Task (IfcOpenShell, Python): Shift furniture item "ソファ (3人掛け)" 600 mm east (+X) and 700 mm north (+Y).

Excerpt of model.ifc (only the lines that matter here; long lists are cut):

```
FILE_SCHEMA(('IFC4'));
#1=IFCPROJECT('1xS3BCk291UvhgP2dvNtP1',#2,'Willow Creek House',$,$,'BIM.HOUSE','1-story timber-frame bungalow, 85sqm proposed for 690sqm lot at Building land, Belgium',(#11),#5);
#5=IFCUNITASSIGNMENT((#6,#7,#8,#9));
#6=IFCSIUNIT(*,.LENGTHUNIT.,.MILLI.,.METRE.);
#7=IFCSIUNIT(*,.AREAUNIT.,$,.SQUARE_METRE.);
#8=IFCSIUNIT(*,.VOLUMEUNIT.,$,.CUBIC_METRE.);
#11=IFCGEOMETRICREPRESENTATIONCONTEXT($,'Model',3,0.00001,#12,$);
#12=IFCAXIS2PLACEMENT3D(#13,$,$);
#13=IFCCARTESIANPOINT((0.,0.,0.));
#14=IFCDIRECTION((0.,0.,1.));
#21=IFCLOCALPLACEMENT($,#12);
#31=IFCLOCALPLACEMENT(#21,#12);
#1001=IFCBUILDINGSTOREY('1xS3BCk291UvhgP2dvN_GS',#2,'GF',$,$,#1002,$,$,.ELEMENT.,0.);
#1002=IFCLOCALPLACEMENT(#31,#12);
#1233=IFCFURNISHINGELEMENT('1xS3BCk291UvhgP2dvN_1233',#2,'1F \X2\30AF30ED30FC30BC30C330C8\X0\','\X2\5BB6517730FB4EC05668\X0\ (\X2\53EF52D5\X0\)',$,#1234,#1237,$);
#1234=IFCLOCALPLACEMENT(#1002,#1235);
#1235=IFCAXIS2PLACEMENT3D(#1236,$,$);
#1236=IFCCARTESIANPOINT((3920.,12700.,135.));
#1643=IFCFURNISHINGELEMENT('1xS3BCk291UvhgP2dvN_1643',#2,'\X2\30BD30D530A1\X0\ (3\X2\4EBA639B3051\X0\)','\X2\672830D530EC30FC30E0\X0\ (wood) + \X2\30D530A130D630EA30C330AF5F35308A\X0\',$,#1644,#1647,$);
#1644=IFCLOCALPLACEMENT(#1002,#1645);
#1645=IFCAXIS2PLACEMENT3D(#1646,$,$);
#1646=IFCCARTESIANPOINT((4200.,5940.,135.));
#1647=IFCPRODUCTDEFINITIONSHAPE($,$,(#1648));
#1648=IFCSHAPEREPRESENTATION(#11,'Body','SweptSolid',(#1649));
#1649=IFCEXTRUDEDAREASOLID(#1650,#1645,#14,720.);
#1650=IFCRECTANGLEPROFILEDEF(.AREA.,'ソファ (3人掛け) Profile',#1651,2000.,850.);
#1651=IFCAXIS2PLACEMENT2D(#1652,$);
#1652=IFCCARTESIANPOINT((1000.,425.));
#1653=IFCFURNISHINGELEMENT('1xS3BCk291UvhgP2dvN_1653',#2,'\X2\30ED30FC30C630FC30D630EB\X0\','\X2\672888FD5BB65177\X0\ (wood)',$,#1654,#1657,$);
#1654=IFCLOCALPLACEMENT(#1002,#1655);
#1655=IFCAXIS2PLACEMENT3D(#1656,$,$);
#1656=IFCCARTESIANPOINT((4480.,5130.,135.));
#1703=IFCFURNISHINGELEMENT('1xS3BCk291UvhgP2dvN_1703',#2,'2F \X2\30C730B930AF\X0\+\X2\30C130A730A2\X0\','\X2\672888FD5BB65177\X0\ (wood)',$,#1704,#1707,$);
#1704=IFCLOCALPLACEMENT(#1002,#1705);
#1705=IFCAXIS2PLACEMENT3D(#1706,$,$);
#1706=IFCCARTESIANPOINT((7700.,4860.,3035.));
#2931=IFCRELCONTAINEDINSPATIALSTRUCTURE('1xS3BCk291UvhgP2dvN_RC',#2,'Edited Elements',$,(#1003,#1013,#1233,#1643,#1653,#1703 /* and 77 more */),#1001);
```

```python
import ifcopenshell
import ifcopenshell.api.geometry
import ifcopenshell.util.placement

model = ifcopenshell.open("model.ifc")

item = model.by_id(1643)
matrix = ifcopenshell.util.placement.get_local_placement(item.ObjectPlacement)
matrix[0, 3] += 600.0
matrix[1, 3] += 700.0
ifcopenshell.api.geometry.edit_object_placement(model, product=item, matrix=matrix, is_si=False)

print(ifcopenshell.util.placement.get_local_placement(item.ObjectPlacement).round(3) + 0.0)

model.write("model_v2.ifc")
```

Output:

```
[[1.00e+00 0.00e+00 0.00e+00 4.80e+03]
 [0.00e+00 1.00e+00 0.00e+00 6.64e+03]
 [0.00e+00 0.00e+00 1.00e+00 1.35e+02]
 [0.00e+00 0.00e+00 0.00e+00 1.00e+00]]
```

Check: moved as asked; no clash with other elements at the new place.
